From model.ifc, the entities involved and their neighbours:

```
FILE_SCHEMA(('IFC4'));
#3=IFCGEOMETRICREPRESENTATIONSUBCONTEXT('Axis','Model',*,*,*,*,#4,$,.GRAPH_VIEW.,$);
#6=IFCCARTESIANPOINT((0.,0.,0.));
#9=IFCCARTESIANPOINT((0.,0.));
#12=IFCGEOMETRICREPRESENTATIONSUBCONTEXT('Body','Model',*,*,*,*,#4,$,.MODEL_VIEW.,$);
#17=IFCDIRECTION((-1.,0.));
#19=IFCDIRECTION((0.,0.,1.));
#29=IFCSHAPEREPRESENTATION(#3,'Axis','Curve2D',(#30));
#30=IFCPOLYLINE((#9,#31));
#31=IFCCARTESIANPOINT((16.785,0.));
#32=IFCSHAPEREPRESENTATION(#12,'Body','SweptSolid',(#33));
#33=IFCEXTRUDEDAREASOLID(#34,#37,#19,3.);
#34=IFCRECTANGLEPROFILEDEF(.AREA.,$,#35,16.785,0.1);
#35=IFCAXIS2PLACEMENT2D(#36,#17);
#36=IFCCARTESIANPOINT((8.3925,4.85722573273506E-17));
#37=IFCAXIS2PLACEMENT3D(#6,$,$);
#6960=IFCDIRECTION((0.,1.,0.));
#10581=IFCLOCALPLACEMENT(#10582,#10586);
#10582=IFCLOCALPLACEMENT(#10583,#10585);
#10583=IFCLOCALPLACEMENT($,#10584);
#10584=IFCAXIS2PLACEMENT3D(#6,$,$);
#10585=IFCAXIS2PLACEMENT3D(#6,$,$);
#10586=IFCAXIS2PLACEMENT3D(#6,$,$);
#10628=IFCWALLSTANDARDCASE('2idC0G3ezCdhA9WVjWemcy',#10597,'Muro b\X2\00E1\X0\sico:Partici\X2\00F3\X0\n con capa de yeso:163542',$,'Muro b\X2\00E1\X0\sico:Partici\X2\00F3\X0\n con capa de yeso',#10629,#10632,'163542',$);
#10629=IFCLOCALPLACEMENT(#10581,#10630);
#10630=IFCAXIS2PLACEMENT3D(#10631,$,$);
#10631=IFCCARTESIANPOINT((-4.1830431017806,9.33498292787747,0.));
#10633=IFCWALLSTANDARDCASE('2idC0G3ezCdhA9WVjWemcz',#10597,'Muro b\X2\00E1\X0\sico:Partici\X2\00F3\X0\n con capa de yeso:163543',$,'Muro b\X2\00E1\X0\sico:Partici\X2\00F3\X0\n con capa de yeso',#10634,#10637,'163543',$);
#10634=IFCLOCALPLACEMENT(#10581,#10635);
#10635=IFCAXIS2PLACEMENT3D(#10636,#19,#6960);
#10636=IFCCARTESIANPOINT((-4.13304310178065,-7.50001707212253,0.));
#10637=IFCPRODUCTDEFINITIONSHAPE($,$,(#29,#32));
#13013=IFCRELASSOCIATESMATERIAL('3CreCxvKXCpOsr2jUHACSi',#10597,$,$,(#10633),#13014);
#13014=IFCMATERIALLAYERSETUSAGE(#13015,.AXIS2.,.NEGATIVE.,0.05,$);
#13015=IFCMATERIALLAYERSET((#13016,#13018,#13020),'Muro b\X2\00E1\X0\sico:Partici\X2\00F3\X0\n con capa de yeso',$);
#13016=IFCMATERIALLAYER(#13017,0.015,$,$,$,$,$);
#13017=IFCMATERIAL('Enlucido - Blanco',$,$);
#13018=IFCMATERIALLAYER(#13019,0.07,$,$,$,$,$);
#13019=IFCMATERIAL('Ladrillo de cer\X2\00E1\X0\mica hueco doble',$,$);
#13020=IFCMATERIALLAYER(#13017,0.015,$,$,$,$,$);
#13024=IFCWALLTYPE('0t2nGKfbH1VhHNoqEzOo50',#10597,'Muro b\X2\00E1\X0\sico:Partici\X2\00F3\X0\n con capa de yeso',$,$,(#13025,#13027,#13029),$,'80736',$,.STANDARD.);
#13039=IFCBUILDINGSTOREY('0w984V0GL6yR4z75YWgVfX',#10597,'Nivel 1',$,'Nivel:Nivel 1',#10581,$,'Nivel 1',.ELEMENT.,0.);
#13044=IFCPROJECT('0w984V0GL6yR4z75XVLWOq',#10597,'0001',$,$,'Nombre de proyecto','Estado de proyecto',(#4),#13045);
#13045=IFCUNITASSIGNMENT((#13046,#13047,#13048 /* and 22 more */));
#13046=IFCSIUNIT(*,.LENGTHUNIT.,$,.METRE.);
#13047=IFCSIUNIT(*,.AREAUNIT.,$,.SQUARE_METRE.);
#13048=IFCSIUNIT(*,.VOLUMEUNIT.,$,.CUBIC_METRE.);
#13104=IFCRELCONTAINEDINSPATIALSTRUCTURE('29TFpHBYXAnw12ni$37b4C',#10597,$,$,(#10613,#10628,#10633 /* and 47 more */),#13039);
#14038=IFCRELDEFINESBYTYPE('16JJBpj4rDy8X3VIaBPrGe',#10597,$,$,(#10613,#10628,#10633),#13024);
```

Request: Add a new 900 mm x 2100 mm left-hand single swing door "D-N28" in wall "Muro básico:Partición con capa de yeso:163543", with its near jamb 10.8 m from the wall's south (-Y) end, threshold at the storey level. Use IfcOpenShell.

```python
import numpy as np
import ifcopenshell
import ifcopenshell.api.feature
import ifcopenshell.api.geometry
import ifcopenshell.api.root
import ifcopenshell.api.spatial
import ifcopenshell.geom
import ifcopenshell.util.element
import ifcopenshell.util.placement
import ifcopenshell.util.representation
import ifcopenshell.util.shape
import ifcopenshell.util.unit

model = ifcopenshell.open("model.ifc")
unit_scale = ifcopenshell.util.unit.calculate_unit_scale(model)
settings = ifcopenshell.geom.settings()


def volume(element):
    """Net volume in cubic metres, openings subtracted."""
    shape = ifcopenshell.geom.create_shape(settings, element)
    return ifcopenshell.util.shape.get_volume(shape.geometry)


wall = model.by_id(10633)
storey = ifcopenshell.util.element.get_container(wall, ifc_class="IfcBuildingStorey")
context = ifcopenshell.util.representation.get_context(model, "Model", "Body", "MODEL_VIEW")
before = volume(wall)

width, height, from_end, sill = 0.9, 2.1, 10.8, 0.0  # metres

# The wall runs along its own X axis, and the end named is its -X end.
wall_shape = ifcopenshell.geom.create_shape(settings, wall)
x, y, z = ifcopenshell.util.shape.get_vertices(wall_shape.geometry).T
start = x.min() + from_end
face, thickness = float(y.min()), float(y.max() - y.min())
wall_matrix = ifcopenshell.util.placement.get_local_placement(wall.ObjectPlacement)
level = ifcopenshell.util.placement.get_local_placement(storey.ObjectPlacement)[2, 3]


def in_wall(x, y):
    """Placement at x, y metres in the wall's axes, at sill height."""
    matrix = wall_matrix.copy()
    matrix[:, 3] = wall_matrix @ np.array([x / unit_scale, y / unit_scale, 0.0, 1.0])
    matrix[2, 3] = level + sill / unit_scale
    return matrix


# Opening: a box that overshoots both wall faces by 50 mm.
opening = ifcopenshell.api.root.create_entity(model, ifc_class="IfcOpeningElement", predefined_type="OPENING")
box = ifcopenshell.api.geometry.add_wall_representation(
    model, context=context, length=width, height=height, thickness=thickness + 0.1
)
ifcopenshell.api.geometry.assign_representation(model, product=opening, representation=box)
ifcopenshell.api.geometry.edit_object_placement(model, product=opening, matrix=in_wall(start, face - 0.05), is_si=False)
ifcopenshell.api.feature.add_feature(model, feature=opening, element=wall)

door = ifcopenshell.api.root.create_entity(model, ifc_class="IfcDoor", name="D-N28", predefined_type="DOOR")
door.OverallWidth, door.OverallHeight = width / unit_scale, height / unit_scale
door.OperationType = "SINGLE_SWING_LEFT"
body = ifcopenshell.api.geometry.add_door_representation(
    model,
    context=context,
    overall_width=door.OverallWidth,
    overall_height=door.OverallHeight,
    operation_type="SINGLE_SWING_LEFT",
    lining_properties={"LiningDepth": thickness / unit_scale, "ThresholdDepth": thickness / unit_scale},
)
ifcopenshell.api.geometry.assign_representation(model, product=door, representation=body)
ifcopenshell.api.spatial.assign_container(model, products=[door], relating_structure=storey)
ifcopenshell.api.feature.add_filling(model, opening=opening, element=door)

# The lining spans the wall, so the door starts at the wall face.
ifcopenshell.api.geometry.edit_object_placement(model, product=door, matrix=in_wall(start, face), is_si=False)

after = volume(wall)

print(f"wall volume {before:.3f} -> {after:.3f} m3")

model.write("model-out.ifc")
```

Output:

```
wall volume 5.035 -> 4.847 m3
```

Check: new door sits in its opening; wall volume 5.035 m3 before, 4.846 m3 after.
